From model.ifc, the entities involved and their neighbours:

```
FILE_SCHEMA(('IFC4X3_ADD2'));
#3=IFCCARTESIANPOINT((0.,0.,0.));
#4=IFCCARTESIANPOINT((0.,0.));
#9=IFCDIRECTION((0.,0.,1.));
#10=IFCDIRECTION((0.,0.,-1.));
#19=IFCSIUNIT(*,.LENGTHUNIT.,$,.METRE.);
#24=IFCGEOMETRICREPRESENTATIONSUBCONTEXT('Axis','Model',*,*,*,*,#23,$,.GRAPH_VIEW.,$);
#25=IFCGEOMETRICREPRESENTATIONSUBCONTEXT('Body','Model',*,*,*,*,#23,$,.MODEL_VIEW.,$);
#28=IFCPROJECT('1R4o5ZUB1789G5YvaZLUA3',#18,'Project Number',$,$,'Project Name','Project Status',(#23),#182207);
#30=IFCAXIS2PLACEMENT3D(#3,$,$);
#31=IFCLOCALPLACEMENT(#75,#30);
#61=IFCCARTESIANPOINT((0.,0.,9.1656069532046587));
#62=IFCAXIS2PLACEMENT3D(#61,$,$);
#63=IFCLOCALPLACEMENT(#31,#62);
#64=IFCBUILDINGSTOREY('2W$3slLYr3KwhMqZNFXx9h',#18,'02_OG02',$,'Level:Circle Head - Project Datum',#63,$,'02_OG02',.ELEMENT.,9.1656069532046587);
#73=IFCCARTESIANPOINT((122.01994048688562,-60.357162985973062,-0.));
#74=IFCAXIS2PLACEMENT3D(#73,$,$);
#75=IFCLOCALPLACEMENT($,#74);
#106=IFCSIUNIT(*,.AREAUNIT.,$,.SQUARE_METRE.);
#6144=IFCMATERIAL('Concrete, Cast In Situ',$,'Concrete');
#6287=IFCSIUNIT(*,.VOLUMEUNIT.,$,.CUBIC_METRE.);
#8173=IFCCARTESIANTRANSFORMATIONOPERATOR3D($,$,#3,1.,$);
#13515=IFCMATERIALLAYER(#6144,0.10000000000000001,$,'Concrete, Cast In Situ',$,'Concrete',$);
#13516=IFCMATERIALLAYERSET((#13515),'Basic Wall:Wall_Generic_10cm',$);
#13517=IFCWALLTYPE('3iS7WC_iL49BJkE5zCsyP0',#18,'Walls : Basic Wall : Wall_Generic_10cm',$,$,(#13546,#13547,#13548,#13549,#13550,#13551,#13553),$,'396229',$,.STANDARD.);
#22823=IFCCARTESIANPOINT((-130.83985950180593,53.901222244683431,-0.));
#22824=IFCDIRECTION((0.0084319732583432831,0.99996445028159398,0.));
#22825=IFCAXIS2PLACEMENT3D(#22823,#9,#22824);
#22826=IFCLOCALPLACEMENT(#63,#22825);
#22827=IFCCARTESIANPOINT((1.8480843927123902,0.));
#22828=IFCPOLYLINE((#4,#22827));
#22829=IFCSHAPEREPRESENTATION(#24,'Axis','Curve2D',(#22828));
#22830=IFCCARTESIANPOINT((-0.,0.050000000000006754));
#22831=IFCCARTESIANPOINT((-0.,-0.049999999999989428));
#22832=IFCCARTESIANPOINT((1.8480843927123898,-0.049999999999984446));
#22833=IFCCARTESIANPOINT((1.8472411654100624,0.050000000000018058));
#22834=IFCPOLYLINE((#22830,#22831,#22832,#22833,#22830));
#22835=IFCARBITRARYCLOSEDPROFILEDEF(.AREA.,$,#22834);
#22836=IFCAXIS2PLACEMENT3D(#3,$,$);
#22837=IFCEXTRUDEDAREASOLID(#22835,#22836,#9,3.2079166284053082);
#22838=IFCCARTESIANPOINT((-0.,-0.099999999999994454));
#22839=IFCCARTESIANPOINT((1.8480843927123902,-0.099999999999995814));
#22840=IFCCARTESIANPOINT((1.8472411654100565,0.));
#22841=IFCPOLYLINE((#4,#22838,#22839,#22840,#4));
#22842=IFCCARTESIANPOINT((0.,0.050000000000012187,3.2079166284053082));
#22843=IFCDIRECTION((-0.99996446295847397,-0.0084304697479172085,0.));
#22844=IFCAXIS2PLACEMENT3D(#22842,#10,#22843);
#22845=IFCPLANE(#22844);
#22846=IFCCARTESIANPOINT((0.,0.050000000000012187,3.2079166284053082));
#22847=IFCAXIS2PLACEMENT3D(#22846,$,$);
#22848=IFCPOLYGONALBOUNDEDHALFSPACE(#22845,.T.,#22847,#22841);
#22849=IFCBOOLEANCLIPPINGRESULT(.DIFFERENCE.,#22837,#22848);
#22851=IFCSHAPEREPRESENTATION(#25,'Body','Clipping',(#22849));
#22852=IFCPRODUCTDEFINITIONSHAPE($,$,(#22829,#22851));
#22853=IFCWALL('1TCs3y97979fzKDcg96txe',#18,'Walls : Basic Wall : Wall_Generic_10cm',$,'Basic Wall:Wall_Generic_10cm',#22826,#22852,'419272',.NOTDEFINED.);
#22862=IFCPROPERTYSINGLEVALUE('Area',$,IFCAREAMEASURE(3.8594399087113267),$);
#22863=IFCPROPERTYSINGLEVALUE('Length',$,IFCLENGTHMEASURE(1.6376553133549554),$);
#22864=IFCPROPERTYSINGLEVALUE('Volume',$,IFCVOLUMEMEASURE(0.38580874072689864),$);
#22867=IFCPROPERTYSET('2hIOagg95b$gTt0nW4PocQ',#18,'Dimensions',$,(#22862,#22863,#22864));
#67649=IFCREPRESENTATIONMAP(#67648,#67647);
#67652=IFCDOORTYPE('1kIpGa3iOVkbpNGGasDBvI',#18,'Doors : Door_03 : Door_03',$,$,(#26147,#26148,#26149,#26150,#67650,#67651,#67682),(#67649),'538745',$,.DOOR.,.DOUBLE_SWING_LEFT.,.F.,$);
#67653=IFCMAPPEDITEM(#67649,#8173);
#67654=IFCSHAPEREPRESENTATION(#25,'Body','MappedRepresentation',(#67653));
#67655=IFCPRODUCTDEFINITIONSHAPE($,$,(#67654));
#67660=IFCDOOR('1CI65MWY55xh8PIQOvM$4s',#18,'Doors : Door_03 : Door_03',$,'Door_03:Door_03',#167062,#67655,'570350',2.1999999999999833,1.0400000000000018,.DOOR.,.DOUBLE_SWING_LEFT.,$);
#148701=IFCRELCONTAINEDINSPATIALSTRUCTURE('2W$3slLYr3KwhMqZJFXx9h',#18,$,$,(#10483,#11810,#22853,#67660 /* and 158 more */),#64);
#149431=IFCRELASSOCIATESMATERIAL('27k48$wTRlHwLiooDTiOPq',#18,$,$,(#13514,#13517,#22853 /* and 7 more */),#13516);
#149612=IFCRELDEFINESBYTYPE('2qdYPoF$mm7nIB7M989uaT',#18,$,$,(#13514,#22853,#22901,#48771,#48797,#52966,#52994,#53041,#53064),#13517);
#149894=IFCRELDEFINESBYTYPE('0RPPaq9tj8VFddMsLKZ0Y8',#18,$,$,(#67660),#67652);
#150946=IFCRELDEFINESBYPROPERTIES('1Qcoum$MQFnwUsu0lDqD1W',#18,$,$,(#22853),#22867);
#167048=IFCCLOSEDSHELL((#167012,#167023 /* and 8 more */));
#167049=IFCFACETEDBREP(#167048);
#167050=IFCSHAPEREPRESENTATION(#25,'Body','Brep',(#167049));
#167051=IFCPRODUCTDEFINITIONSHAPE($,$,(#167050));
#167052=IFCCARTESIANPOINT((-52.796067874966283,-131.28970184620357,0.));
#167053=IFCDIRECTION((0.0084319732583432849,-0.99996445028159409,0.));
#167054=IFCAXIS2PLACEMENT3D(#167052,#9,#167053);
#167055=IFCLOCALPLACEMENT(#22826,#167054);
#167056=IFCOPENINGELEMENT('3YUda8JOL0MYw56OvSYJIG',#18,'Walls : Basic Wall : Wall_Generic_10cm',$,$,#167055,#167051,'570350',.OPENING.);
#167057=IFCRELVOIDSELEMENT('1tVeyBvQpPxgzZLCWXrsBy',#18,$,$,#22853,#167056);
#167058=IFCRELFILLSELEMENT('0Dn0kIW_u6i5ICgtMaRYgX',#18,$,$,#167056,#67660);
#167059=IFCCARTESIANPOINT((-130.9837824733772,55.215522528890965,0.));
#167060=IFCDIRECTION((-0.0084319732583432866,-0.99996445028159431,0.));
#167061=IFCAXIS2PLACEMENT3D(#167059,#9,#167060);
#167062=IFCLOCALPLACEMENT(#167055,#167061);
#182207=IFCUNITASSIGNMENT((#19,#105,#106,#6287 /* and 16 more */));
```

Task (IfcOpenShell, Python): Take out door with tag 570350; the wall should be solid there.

```python
import ifcopenshell
import ifcopenshell.api.feature
import ifcopenshell.api.pset
import ifcopenshell.api.root
import ifcopenshell.geom
import ifcopenshell.util.element
import ifcopenshell.util.shape
import ifcopenshell.util.unit

model = ifcopenshell.open("model.ifc")
area_scale = ifcopenshell.util.unit.calculate_unit_scale(model, "AREAUNIT")
volume_scale = ifcopenshell.util.unit.calculate_unit_scale(model, "VOLUMEUNIT")
settings = ifcopenshell.geom.settings()


def volume(element):
    """Net volume in cubic metres, openings subtracted."""
    shape = ifcopenshell.geom.create_shape(settings, element)
    return ifcopenshell.util.shape.get_volume(shape.geometry)


door = model.by_id(67660)
opening = door.FillsVoids[0].RelatingOpeningElement
wall = opening.VoidsElements[0].RelatingBuildingElement
before = volume(wall)

ifcopenshell.api.root.remove_product(model, product=door)
ifcopenshell.api.feature.remove_feature(model, feature=opening)

after = volume(wall)
thickness = 0.1  # wall thickness in metres

# Update the wall's stored quantities.
pset = model.by_id(ifcopenshell.util.element.get_pset(wall, "Dimensions", should_inherit=False)["id"])
ifcopenshell.api.pset.edit_pset(model, pset=pset, properties={
    "Area": model.create_entity("IfcAreaMeasure", after / thickness / area_scale),
    "Volume": model.create_entity("IfcVolumeMeasure", after / volume_scale),
})

print(f"wall volume {before:.3f} -> {after:.3f} m3")

model.write("model_v2.ifc")
```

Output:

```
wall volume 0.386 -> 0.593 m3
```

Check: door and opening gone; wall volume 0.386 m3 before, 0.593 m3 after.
